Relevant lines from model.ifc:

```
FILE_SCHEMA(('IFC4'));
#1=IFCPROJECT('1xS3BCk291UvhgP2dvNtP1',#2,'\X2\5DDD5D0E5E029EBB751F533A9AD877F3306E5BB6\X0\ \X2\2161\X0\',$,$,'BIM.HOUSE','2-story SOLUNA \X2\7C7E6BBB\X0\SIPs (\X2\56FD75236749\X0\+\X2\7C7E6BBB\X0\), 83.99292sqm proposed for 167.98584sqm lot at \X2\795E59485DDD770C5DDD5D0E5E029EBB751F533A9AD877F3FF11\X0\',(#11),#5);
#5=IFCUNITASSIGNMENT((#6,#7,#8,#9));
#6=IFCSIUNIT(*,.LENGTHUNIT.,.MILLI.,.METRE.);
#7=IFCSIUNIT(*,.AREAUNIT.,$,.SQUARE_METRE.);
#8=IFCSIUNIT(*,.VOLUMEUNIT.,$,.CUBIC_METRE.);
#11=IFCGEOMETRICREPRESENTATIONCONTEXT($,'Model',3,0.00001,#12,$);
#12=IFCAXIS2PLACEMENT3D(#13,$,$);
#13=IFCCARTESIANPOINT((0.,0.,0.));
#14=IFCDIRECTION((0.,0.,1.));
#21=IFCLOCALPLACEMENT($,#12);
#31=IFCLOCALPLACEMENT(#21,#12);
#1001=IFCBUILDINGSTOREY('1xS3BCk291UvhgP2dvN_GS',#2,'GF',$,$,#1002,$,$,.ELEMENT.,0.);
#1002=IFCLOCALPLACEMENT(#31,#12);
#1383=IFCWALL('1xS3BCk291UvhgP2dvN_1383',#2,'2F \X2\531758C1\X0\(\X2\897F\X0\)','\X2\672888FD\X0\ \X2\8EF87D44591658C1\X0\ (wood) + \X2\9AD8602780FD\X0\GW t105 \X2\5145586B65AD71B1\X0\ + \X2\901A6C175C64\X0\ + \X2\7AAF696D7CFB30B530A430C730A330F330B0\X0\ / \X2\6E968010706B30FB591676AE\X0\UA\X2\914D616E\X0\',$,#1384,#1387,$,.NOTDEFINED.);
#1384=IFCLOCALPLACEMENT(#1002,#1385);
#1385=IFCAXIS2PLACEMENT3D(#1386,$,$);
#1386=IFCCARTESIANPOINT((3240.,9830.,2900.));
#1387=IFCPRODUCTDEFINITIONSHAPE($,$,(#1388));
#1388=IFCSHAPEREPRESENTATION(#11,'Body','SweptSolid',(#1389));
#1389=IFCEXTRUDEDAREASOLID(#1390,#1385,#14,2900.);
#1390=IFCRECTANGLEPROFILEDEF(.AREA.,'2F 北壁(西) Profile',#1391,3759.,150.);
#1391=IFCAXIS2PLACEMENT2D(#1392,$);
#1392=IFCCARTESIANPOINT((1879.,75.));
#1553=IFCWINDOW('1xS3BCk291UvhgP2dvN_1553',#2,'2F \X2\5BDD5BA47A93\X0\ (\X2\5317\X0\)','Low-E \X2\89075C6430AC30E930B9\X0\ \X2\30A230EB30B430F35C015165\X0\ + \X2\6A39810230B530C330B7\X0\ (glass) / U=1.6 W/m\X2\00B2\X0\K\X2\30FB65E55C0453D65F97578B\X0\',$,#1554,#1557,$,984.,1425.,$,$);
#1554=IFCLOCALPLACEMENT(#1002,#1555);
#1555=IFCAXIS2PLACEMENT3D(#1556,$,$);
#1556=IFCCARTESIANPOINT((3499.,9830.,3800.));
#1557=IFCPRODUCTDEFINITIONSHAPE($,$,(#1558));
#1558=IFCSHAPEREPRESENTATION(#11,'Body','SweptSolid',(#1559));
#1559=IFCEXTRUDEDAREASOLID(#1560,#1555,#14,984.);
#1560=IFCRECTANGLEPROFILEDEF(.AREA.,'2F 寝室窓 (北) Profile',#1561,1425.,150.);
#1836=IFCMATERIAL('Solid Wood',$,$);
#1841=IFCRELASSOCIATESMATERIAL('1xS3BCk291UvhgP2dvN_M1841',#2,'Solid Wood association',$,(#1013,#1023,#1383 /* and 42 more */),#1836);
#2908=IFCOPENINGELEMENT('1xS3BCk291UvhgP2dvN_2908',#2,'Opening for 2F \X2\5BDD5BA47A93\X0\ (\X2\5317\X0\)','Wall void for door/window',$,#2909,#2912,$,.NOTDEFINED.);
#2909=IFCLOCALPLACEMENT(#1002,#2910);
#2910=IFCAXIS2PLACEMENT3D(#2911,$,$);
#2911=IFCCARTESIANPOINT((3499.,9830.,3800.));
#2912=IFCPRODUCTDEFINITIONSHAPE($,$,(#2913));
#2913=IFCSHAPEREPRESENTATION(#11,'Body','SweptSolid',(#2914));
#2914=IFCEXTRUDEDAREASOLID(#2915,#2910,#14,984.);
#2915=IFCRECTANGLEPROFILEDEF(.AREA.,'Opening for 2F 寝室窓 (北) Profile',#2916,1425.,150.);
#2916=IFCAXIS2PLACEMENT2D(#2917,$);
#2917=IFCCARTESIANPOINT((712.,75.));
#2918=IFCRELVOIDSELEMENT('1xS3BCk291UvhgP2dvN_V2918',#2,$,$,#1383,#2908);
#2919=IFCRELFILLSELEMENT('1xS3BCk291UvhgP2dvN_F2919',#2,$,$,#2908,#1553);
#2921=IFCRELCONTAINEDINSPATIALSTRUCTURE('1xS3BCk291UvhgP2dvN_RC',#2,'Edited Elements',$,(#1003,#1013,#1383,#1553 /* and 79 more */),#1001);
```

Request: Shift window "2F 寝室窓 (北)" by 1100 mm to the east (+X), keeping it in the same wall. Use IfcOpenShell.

```python
import ifcopenshell
import ifcopenshell.api.geometry
import ifcopenshell.util.placement
import ifcopenshell.util.unit

model = ifcopenshell.open("model.ifc")
unit_scale = ifcopenshell.util.unit.calculate_unit_scale(model)

window = model.by_guid("1xS3BCk291UvhgP2dvN_1553")
opening = window.FillsVoids[0].RelatingOpeningElement
wall = opening.VoidsElements[0].RelatingBuildingElement

wall_matrix = ifcopenshell.util.placement.get_local_placement(wall.ObjectPlacement)
shift = wall_matrix[:3, 0] * 1.1 / unit_scale
before = ifcopenshell.util.placement.get_local_placement(window.ObjectPlacement)[:3, 3].copy()

# The window is not placed relative to its opening, so move both.
for product in (opening, window):
    matrix = ifcopenshell.util.placement.get_local_placement(product.ObjectPlacement)
    matrix[:3, 3] += shift
    ifcopenshell.api.geometry.edit_object_placement(model, product=product, matrix=matrix, is_si=False)

after = ifcopenshell.util.placement.get_local_placement(window.ObjectPlacement)[:3, 3]
print("window moved by", (after - before).round(3) + 0.0)

model.write("model-out.ifc")
```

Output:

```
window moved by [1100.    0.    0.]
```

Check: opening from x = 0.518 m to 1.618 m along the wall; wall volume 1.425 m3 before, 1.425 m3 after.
